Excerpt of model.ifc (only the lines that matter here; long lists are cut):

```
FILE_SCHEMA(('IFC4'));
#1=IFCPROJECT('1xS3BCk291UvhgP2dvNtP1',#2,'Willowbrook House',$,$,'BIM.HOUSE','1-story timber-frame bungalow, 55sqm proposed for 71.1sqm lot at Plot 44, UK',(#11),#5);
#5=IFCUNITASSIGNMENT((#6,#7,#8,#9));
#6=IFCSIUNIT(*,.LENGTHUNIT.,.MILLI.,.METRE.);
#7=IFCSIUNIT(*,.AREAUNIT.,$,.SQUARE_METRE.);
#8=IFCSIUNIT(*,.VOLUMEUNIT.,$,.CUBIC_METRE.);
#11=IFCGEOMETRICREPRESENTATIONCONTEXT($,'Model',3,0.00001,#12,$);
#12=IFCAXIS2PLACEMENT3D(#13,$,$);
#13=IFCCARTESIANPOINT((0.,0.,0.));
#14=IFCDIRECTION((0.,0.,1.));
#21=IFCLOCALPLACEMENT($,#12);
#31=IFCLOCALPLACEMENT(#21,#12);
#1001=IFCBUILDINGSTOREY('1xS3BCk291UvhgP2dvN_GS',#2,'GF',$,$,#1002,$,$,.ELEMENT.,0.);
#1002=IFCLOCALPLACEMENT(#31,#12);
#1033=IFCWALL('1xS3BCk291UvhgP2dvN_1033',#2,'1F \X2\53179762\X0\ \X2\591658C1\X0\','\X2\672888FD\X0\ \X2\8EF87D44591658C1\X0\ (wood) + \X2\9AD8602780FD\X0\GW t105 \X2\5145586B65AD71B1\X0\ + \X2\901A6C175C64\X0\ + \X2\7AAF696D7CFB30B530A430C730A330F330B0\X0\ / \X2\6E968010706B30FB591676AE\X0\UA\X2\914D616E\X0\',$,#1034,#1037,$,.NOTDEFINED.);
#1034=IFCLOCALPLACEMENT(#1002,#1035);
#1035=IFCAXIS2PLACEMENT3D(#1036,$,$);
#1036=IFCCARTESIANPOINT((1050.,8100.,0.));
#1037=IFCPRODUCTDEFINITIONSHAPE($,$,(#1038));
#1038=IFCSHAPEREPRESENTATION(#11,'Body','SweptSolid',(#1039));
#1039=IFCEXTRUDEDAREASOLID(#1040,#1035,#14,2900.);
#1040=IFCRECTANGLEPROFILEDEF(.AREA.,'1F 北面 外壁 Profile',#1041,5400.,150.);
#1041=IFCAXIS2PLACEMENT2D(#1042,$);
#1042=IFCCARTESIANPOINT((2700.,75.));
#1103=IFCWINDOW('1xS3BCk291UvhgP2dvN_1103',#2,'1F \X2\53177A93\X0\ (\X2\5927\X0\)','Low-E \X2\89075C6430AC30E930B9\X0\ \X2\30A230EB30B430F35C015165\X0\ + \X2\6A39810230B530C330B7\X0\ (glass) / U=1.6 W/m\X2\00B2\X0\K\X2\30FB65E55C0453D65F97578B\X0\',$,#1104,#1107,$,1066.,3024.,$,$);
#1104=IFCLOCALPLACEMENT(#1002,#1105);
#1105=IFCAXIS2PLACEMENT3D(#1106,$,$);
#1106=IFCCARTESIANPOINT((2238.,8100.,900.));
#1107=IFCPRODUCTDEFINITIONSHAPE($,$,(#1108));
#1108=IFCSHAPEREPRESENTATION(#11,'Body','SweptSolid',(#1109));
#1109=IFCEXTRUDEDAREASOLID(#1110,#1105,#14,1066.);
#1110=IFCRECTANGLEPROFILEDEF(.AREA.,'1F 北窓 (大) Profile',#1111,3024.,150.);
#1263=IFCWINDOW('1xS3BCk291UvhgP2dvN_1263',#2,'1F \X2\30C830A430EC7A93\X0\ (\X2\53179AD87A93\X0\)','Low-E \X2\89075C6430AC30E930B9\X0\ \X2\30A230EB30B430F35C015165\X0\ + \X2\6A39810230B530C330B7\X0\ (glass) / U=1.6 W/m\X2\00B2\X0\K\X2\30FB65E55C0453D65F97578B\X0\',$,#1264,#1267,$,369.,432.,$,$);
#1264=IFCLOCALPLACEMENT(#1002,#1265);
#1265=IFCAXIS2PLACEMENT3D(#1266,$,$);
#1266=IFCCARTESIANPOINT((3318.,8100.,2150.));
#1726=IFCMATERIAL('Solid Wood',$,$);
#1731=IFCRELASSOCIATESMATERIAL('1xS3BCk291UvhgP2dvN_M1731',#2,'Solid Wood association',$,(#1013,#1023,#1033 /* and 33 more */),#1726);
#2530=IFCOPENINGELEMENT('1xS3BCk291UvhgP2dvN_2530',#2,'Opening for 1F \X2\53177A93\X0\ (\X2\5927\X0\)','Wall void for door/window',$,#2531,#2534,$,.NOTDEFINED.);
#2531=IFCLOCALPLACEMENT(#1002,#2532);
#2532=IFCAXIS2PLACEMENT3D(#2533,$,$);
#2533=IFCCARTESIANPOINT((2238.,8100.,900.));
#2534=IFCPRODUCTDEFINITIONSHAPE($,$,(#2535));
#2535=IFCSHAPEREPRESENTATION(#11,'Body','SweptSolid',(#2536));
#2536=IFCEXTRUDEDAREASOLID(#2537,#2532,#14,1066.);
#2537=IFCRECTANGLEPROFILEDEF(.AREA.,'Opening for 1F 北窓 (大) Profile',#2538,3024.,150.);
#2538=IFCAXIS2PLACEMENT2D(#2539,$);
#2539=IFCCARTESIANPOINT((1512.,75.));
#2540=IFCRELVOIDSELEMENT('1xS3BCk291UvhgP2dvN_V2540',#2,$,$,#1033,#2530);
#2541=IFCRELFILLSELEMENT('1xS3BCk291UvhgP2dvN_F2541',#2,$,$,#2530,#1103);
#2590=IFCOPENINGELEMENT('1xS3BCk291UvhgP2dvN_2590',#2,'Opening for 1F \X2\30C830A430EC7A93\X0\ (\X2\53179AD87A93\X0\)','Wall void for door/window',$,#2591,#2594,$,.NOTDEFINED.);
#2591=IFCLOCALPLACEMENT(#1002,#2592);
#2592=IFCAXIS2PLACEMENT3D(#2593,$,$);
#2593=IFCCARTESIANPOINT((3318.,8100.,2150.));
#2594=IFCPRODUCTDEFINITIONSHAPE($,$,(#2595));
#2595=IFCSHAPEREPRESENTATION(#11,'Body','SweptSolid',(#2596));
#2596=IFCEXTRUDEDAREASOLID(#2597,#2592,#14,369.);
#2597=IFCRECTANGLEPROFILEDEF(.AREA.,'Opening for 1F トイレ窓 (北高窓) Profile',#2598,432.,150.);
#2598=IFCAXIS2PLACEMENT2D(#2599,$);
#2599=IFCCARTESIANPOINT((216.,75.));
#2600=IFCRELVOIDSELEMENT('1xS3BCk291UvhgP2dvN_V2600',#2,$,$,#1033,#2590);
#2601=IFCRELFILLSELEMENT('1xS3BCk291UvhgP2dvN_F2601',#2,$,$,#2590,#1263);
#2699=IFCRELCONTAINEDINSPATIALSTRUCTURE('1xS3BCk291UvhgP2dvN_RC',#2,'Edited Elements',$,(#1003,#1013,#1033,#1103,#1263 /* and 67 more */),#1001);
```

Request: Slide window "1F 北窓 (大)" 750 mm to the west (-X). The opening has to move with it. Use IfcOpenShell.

```python
import ifcopenshell
import ifcopenshell.api.geometry
import ifcopenshell.util.placement
import ifcopenshell.util.unit

model = ifcopenshell.open("model.ifc")
unit_scale = ifcopenshell.util.unit.calculate_unit_scale(model)

window = model.by_guid("1xS3BCk291UvhgP2dvN_1103")
opening = window.FillsVoids[0].RelatingOpeningElement
wall = opening.VoidsElements[0].RelatingBuildingElement

wall_matrix = ifcopenshell.util.placement.get_local_placement(wall.ObjectPlacement)
shift = wall_matrix[:3, 0] * -0.75 / unit_scale
before = ifcopenshell.util.placement.get_local_placement(window.ObjectPlacement)[:3, 3].copy()

# The window is not placed relative to its opening, so move both.
for product in (opening, window):
    matrix = ifcopenshell.util.placement.get_local_placement(product.ObjectPlacement)
    matrix[:3, 3] += shift
    ifcopenshell.api.geometry.edit_object_placement(model, product=product, matrix=matrix, is_si=False)

after = ifcopenshell.util.placement.get_local_placement(window.ObjectPlacement)[:3, 3]
print("window moved by", (after - before).round(3) + 0.0)

model.write("model_v2.ifc")
```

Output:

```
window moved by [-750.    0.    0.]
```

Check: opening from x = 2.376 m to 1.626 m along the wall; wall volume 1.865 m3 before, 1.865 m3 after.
